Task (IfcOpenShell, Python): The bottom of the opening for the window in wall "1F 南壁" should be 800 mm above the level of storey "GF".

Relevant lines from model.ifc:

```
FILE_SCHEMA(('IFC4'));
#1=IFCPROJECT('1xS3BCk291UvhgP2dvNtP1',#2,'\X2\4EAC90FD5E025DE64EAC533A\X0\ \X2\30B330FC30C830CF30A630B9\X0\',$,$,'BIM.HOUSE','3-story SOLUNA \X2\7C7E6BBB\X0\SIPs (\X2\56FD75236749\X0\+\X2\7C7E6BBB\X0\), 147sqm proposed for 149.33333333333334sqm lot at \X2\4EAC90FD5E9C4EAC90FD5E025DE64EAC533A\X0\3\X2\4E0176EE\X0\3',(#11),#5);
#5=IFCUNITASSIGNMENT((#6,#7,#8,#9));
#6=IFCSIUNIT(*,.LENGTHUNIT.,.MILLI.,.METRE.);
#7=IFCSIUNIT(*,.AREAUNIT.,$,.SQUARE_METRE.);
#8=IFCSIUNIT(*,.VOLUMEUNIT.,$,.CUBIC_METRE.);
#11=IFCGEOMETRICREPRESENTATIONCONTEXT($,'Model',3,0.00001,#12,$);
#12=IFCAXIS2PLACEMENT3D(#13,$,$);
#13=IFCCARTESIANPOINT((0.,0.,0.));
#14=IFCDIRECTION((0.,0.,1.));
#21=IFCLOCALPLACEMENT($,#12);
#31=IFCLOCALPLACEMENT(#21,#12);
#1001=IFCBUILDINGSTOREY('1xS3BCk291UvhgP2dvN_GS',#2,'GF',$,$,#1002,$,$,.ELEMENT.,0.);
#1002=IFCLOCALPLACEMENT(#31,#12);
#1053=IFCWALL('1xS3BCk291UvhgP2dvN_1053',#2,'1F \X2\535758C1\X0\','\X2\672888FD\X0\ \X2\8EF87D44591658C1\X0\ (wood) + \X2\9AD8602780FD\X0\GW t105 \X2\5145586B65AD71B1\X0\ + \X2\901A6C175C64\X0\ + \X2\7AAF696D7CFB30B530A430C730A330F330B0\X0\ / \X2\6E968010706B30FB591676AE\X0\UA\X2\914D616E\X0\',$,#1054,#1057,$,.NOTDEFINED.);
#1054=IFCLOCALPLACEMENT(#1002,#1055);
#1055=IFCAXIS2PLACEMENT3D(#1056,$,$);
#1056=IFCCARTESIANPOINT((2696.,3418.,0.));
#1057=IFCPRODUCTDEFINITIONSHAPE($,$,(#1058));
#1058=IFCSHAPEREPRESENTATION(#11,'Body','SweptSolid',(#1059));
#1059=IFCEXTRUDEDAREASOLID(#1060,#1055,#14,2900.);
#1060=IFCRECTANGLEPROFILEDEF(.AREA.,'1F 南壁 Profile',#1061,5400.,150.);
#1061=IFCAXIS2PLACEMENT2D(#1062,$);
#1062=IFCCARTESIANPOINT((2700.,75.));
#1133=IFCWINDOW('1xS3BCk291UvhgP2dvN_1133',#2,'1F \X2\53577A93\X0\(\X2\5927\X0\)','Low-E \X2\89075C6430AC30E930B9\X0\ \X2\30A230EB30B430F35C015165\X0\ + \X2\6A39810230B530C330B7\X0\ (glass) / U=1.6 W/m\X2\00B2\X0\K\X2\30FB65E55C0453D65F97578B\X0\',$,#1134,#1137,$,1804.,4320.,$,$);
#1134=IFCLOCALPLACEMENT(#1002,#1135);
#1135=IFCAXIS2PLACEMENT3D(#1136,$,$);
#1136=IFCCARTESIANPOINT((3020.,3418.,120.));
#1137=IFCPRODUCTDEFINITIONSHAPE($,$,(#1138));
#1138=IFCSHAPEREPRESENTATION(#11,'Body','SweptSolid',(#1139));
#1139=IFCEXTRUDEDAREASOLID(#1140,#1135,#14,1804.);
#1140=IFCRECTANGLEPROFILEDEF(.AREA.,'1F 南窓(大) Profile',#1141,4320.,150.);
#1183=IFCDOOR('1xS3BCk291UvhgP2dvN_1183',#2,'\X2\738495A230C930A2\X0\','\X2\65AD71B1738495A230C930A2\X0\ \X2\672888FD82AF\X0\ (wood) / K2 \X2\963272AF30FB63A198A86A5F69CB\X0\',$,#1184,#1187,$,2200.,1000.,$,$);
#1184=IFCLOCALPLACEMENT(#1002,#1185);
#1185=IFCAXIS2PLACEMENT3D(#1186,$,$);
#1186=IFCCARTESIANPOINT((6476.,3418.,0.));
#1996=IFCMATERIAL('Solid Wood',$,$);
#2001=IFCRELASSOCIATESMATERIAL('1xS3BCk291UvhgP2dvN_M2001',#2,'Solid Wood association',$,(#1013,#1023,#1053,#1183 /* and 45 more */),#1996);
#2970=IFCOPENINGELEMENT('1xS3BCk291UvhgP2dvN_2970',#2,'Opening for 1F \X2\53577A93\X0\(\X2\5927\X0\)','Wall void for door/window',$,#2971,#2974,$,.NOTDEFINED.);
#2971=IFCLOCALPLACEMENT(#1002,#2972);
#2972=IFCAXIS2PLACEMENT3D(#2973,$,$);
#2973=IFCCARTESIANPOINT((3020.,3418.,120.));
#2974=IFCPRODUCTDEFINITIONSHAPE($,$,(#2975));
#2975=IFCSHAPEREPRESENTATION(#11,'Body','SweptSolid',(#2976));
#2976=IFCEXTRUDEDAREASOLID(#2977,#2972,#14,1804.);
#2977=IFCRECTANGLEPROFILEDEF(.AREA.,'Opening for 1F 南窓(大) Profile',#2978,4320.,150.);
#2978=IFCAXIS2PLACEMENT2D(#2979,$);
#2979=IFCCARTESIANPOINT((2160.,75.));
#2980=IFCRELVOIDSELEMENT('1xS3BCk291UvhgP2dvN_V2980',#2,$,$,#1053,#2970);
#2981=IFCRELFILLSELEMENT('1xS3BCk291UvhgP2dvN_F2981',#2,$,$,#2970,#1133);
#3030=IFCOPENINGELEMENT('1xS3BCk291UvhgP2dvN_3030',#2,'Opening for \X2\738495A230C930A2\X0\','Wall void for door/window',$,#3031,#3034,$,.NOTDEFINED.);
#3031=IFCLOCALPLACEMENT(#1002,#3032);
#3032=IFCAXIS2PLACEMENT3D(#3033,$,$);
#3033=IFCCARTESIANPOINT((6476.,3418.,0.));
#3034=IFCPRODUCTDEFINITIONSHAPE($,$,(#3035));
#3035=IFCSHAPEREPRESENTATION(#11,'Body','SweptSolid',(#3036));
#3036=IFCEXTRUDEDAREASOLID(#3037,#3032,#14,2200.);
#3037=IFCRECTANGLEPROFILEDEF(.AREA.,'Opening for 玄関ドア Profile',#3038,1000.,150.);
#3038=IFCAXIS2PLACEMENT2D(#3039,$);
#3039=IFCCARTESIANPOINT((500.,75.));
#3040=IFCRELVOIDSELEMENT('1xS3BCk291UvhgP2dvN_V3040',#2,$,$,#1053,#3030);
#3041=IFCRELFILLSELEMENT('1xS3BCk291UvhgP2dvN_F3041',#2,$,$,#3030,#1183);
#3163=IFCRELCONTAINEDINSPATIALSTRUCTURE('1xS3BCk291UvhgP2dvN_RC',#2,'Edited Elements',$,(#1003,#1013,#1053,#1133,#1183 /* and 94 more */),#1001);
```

```python
import numpy as np
import ifcopenshell
import ifcopenshell.api.geometry
import ifcopenshell.geom
import ifcopenshell.util.element
import ifcopenshell.util.placement
import ifcopenshell.util.shape
import ifcopenshell.util.unit

model = ifcopenshell.open("model.ifc")
unit_scale = ifcopenshell.util.unit.calculate_unit_scale(model)

window = model.by_guid("1xS3BCk291UvhgP2dvN_1133")
opening = window.FillsVoids[0].RelatingOpeningElement
storey = ifcopenshell.util.element.get_container(window, ifc_class="IfcBuildingStorey")
level = ifcopenshell.util.placement.get_local_placement(storey.ObjectPlacement)[2, 3]

# The opening's origin need not be at the sill, so measure its lowest point.
shape = ifcopenshell.geom.create_shape(ifcopenshell.geom.settings(), opening)
bottom = ifcopenshell.util.shape.get_shape_bottom_elevation(shape, shape.geometry) / unit_scale
dz = level + 0.8 / unit_scale - bottom

shift = np.array([0.0, 0.0, dz])
# The window is not placed relative to its opening, so move both.
for product in (opening, window):
    matrix = ifcopenshell.util.placement.get_local_placement(product.ObjectPlacement)
    matrix[:3, 3] += shift
    ifcopenshell.api.geometry.edit_object_placement(model, product=product, matrix=matrix, is_si=False)

print(f"moved by {dz * unit_scale:+.3f} m")

model.write("model-out.ifc")
```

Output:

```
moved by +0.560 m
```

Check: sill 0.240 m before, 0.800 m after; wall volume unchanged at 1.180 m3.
